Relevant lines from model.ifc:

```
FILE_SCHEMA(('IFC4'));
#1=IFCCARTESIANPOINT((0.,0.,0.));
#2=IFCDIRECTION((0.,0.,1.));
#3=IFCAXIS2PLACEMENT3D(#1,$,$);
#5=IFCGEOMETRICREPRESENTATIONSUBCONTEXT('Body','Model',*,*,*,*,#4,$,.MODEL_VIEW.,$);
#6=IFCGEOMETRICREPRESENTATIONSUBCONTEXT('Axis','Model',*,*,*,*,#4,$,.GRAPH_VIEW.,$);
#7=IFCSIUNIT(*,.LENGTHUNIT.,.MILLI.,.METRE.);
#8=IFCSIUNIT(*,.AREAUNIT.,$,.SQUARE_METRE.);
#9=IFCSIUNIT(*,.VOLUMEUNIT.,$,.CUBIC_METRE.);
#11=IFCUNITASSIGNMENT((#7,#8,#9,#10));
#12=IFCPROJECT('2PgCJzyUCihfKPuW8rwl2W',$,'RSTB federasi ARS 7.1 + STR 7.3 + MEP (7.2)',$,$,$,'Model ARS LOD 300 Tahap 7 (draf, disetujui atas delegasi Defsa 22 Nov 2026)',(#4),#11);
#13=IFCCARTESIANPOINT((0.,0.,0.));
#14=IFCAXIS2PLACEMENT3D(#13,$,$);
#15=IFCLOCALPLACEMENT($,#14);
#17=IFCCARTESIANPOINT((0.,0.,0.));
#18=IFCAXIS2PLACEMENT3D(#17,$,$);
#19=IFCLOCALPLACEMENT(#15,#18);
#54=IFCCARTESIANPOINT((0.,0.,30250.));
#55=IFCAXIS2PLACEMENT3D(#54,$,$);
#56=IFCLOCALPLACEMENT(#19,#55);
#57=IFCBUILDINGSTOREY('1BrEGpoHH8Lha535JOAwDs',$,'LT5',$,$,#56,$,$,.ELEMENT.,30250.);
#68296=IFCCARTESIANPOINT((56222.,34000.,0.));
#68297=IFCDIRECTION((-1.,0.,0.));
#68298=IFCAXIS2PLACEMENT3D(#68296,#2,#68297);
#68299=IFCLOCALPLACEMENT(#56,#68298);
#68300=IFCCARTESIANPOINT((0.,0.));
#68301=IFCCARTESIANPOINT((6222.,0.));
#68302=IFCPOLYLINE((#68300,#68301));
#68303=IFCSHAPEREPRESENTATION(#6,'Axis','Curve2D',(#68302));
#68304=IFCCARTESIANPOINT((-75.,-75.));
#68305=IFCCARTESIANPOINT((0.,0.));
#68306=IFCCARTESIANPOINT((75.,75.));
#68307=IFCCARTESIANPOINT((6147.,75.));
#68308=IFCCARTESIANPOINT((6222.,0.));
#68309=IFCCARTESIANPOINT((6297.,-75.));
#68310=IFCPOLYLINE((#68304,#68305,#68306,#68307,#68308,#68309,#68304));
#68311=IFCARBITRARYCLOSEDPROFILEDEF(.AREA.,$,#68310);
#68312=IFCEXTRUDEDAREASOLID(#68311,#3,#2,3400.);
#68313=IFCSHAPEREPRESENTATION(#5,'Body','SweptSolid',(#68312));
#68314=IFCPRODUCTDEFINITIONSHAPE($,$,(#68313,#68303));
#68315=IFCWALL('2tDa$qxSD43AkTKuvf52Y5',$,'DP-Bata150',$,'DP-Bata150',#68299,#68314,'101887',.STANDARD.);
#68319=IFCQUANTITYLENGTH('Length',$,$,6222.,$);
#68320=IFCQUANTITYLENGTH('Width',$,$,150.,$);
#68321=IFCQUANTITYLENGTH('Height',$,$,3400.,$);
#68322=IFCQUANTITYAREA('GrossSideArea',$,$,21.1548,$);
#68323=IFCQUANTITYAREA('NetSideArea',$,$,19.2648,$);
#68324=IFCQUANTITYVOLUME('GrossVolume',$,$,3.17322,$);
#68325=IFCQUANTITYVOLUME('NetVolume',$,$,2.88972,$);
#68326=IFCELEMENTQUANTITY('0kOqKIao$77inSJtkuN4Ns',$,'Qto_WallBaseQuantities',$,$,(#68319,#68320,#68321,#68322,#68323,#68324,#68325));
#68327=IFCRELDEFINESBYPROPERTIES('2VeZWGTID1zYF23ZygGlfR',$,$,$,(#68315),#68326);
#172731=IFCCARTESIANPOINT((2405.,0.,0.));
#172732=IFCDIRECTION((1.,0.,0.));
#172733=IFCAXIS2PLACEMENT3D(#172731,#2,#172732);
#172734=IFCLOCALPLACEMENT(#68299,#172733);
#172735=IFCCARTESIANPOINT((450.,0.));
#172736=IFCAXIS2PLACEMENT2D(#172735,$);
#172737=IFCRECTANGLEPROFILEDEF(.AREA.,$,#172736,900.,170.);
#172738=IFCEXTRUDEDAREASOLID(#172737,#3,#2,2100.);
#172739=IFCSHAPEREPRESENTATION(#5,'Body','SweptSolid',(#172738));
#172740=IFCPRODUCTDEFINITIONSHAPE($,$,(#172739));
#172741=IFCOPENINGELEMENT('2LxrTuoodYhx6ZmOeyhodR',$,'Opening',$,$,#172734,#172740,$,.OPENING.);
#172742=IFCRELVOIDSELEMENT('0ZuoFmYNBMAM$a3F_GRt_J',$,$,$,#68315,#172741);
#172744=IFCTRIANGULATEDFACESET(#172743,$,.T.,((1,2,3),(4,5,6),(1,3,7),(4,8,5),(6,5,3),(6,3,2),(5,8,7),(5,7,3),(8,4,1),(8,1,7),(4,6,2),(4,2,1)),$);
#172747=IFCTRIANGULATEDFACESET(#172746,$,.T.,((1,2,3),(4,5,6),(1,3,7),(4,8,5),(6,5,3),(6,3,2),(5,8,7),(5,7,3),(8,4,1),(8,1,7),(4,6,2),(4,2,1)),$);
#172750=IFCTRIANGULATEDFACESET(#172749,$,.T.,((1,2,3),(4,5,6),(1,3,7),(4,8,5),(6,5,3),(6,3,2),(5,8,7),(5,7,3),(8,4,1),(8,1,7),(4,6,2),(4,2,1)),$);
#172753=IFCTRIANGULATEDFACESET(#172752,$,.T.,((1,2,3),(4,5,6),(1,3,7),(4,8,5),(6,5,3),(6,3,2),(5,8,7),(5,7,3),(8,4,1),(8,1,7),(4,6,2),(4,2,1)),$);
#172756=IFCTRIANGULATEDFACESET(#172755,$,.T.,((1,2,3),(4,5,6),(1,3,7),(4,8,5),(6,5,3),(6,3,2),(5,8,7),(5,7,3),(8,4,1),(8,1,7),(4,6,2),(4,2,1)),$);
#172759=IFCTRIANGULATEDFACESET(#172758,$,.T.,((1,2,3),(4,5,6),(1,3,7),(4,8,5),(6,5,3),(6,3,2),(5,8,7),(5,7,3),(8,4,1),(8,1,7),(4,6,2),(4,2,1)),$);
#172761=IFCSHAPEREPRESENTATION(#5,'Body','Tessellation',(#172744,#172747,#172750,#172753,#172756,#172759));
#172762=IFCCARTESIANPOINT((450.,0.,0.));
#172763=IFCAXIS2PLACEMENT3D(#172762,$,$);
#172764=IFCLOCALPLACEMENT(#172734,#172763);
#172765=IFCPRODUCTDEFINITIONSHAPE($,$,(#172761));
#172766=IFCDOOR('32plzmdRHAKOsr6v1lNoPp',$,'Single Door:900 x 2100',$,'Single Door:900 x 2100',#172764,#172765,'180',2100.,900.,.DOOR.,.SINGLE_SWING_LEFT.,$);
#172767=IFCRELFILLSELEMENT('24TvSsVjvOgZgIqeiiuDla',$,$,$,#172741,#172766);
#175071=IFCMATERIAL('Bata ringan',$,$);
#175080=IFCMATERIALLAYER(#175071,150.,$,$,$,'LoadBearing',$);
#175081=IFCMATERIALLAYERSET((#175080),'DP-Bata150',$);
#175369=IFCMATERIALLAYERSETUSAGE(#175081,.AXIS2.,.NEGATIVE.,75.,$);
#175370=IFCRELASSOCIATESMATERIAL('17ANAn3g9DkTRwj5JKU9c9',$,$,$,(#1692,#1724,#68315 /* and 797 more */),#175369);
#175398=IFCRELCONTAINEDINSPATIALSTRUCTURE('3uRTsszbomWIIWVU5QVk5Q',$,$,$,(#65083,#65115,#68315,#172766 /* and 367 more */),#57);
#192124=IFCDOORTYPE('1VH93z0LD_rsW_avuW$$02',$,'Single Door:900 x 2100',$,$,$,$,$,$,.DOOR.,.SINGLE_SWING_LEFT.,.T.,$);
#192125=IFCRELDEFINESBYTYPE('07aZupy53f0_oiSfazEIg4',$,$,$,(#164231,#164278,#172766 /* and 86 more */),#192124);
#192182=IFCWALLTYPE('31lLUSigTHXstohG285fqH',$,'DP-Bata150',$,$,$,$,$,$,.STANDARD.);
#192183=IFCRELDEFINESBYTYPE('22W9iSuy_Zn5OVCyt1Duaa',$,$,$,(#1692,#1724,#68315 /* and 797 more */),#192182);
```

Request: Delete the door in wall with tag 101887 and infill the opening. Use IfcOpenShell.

```python
import ifcopenshell
import ifcopenshell.api.feature
import ifcopenshell.api.pset
import ifcopenshell.api.root
import ifcopenshell.geom
import ifcopenshell.util.element
import ifcopenshell.util.shape
import ifcopenshell.util.unit

model = ifcopenshell.open("model.ifc")
area_scale = ifcopenshell.util.unit.calculate_unit_scale(model, "AREAUNIT")
volume_scale = ifcopenshell.util.unit.calculate_unit_scale(model, "VOLUMEUNIT")
settings = ifcopenshell.geom.settings()


def volume(element):
    """Net volume in cubic metres, openings subtracted."""
    shape = ifcopenshell.geom.create_shape(settings, element)
    return ifcopenshell.util.shape.get_volume(shape.geometry)


door = model.by_guid("32plzmdRHAKOsr6v1lNoPp")
opening = door.FillsVoids[0].RelatingOpeningElement
wall = opening.VoidsElements[0].RelatingBuildingElement
before = volume(wall)

ifcopenshell.api.root.remove_product(model, product=door)
ifcopenshell.api.feature.remove_feature(model, feature=opening)

after = volume(wall)
thickness = 0.15  # wall thickness in metres

# Update the wall's stored quantities.
qto = model.by_id(ifcopenshell.util.element.get_pset(wall, "Qto_WallBaseQuantities", should_inherit=False)["id"])
ifcopenshell.api.pset.edit_qto(model, qto=qto, properties={
    "NetSideArea": after / thickness / area_scale,
    "NetVolume": after / volume_scale,
})

print(f"wall volume {before:.3f} -> {after:.3f} m3")

model.write("model_updated.ifc")
```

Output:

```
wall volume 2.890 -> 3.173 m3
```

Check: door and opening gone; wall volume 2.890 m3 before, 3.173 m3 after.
